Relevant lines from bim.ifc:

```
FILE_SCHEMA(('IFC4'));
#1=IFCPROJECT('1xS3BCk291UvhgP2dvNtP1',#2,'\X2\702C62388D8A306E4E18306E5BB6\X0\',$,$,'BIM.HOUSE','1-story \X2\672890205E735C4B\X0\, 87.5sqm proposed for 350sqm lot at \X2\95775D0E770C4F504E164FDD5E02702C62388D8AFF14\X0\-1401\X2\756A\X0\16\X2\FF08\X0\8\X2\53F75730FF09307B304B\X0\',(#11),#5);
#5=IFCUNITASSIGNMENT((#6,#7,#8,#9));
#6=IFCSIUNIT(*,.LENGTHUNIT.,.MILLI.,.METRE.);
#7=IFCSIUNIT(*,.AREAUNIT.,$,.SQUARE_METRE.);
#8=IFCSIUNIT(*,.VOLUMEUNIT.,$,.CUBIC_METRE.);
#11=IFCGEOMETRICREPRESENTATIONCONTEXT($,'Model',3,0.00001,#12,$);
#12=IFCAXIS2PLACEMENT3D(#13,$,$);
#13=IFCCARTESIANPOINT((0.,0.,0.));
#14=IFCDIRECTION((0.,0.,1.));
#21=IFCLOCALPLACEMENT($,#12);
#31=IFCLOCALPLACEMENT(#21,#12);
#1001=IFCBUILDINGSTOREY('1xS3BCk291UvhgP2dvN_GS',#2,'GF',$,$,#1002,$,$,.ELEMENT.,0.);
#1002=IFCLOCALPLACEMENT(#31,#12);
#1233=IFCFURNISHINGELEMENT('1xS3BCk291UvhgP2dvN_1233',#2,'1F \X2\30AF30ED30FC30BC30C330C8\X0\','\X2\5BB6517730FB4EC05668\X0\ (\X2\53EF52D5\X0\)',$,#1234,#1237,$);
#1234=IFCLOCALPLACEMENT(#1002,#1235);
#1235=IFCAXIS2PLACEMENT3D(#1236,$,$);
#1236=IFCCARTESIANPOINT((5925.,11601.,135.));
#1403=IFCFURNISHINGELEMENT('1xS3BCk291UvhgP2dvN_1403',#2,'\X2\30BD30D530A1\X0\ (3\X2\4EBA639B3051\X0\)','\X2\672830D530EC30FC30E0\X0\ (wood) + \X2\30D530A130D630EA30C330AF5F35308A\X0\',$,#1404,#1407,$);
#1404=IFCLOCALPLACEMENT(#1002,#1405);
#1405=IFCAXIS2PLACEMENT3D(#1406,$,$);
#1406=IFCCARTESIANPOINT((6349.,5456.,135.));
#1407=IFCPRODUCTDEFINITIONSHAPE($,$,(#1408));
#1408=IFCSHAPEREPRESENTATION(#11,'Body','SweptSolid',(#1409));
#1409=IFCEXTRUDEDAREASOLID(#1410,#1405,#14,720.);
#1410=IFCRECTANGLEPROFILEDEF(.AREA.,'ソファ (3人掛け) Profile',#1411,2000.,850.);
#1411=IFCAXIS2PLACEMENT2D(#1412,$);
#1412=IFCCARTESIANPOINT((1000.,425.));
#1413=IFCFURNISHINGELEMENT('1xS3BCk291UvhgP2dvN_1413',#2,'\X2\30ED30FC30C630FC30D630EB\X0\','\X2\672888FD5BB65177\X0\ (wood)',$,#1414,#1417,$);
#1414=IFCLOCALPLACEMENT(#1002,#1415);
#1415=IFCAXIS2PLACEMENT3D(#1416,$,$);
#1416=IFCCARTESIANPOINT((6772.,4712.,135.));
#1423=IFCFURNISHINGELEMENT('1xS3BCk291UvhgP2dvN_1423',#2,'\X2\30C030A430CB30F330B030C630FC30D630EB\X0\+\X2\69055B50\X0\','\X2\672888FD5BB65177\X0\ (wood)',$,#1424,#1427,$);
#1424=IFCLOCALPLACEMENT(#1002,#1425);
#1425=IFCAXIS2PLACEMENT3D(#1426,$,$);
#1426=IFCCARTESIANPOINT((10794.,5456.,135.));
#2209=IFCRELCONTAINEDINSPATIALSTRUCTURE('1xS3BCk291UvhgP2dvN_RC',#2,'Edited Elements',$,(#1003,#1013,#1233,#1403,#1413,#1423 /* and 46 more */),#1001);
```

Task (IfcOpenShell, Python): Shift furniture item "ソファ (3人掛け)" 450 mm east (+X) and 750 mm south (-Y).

```python
import ifcopenshell
import ifcopenshell.api.geometry
import ifcopenshell.util.placement

model = ifcopenshell.open("bim.ifc")

item = model.by_id(1403)
matrix = ifcopenshell.util.placement.get_local_placement(item.ObjectPlacement)
matrix[0, 3] += 450.0
matrix[1, 3] -= 750.0
ifcopenshell.api.geometry.edit_object_placement(model, product=item, matrix=matrix, is_si=False)

print(ifcopenshell.util.placement.get_local_placement(item.ObjectPlacement).round(3) + 0.0)

model.write("bim_v2.ifc")
```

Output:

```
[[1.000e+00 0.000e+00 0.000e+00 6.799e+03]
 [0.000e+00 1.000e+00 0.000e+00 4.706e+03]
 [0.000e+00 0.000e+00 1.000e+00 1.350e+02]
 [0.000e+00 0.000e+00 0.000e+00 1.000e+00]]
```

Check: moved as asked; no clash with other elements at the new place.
